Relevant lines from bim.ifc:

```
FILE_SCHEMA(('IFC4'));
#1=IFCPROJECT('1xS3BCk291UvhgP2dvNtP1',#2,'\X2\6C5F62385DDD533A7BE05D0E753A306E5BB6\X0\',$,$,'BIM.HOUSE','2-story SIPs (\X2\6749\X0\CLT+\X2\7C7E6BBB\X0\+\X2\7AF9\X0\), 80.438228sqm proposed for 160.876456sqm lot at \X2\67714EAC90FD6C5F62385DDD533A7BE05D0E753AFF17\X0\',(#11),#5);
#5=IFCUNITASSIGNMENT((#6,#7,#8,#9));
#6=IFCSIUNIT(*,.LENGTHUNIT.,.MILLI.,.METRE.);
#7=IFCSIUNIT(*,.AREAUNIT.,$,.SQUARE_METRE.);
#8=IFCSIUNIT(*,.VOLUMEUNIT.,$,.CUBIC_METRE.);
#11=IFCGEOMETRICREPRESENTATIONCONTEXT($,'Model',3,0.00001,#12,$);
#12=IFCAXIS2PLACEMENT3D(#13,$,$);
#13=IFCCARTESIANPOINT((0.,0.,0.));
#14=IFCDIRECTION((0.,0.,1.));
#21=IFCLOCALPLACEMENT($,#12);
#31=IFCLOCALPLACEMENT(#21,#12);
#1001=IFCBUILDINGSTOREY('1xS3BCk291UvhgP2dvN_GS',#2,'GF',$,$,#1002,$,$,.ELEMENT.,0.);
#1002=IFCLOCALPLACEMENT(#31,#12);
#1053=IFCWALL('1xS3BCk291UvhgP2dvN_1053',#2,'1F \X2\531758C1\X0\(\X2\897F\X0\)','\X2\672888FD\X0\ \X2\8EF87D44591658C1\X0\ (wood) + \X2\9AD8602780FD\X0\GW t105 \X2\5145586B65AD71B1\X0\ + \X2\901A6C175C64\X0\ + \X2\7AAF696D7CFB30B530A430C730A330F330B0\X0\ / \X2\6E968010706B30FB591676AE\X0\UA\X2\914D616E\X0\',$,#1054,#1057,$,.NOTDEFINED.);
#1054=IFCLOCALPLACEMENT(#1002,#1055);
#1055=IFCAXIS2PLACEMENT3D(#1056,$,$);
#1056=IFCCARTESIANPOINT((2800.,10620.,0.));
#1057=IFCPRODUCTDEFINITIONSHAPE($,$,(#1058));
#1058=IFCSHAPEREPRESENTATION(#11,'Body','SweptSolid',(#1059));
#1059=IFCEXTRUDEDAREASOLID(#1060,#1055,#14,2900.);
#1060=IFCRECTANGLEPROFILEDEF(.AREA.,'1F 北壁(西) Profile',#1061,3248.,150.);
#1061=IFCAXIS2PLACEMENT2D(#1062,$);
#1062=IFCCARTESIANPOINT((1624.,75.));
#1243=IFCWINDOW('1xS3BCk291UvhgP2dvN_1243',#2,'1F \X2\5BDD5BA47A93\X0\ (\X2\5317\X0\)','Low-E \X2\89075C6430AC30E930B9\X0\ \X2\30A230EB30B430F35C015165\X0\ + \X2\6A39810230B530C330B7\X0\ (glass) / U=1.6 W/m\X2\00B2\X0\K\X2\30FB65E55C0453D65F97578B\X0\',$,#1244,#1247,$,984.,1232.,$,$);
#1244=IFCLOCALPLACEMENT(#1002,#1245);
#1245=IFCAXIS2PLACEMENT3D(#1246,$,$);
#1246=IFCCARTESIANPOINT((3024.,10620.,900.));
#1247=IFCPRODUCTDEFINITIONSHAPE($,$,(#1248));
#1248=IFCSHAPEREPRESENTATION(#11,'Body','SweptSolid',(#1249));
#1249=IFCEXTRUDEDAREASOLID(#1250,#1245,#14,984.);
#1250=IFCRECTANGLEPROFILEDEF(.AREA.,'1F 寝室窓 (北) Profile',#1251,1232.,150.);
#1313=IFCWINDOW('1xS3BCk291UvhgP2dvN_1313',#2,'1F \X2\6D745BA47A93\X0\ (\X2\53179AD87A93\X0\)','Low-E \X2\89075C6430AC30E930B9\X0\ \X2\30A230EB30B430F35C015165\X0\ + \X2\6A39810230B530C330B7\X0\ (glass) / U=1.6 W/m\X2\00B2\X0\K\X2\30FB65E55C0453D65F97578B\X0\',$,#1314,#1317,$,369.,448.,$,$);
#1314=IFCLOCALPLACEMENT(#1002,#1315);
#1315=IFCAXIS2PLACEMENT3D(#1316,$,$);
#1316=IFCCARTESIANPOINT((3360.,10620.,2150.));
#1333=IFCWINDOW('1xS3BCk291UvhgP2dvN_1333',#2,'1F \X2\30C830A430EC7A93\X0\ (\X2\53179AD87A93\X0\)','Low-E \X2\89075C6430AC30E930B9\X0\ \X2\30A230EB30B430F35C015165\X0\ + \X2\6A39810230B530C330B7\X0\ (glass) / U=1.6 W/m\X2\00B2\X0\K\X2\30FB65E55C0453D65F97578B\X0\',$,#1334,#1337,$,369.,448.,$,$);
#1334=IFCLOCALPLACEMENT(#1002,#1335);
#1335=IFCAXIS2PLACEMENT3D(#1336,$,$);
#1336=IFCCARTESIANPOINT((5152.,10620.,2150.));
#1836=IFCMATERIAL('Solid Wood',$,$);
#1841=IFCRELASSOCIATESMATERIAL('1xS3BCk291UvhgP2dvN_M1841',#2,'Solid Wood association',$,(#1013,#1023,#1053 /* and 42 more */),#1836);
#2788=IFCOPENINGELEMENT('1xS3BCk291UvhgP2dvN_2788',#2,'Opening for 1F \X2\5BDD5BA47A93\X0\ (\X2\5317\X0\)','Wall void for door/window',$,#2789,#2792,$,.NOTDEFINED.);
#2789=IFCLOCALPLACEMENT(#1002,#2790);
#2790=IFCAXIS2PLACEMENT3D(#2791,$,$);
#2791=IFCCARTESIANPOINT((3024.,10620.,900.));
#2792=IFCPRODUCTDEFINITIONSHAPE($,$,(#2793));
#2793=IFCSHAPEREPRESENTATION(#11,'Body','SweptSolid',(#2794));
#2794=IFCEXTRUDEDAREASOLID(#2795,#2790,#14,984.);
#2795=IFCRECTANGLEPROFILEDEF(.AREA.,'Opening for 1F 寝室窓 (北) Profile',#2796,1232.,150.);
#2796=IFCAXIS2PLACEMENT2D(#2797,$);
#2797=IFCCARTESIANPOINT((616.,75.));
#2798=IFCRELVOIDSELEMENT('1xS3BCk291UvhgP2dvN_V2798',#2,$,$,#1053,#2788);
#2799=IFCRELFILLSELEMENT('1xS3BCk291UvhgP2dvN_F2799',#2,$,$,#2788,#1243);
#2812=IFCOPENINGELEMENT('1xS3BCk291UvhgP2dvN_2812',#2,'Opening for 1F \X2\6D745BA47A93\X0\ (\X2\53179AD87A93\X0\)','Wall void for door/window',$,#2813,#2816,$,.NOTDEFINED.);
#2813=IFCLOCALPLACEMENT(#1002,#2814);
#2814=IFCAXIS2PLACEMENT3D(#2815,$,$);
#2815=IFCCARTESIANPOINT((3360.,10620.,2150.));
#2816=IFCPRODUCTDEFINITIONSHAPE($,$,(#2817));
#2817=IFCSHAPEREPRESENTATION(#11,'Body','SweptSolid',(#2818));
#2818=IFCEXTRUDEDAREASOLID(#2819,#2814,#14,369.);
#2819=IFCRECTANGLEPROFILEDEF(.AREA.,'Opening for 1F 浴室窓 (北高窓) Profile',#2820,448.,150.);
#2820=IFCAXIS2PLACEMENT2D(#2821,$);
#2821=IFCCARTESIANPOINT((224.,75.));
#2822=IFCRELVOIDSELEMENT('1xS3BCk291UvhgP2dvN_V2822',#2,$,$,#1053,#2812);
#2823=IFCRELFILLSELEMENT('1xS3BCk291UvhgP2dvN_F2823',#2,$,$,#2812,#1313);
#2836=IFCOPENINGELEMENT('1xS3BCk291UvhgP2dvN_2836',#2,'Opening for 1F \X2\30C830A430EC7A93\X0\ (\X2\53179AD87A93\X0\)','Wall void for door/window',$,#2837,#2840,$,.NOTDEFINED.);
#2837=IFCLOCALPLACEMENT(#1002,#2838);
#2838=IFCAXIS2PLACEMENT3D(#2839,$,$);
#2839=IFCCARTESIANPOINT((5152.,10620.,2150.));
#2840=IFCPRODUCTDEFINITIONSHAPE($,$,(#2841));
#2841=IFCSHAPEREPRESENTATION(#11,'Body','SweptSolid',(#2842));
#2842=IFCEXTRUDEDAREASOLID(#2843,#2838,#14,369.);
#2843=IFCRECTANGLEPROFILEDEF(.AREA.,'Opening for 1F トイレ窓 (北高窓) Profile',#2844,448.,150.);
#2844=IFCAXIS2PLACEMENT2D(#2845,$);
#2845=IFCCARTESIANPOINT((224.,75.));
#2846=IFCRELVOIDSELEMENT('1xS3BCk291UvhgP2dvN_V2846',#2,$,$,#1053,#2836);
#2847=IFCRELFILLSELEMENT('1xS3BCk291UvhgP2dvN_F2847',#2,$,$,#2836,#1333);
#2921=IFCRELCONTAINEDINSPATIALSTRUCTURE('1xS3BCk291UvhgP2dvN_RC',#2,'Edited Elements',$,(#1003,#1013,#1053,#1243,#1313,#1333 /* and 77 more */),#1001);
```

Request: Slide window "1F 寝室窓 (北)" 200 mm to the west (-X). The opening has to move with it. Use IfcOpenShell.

```python
import ifcopenshell
import ifcopenshell.api.geometry
import ifcopenshell.util.placement

model = ifcopenshell.open("bim.ifc")

window = model.by_guid("1xS3BCk291UvhgP2dvN_1243")
opening = window.FillsVoids[0].RelatingOpeningElement
wall = opening.VoidsElements[0].RelatingBuildingElement

wall_matrix = ifcopenshell.util.placement.get_local_placement(wall.ObjectPlacement)
shift = wall_matrix[:3, 0] * -200.0
before = ifcopenshell.util.placement.get_local_placement(window.ObjectPlacement)[:3, 3].copy()

# The window is not placed relative to its opening, so move both.
for product in (opening, window):
    matrix = ifcopenshell.util.placement.get_local_placement(product.ObjectPlacement)
    matrix[:3, 3] += shift
    ifcopenshell.api.geometry.edit_object_placement(model, product=product, matrix=matrix, is_si=False)

after = ifcopenshell.util.placement.get_local_placement(window.ObjectPlacement)[:3, 3]
print("window moved by", (after - before).round(3) + 0.0)

model.write("bim_rev.ifc")
```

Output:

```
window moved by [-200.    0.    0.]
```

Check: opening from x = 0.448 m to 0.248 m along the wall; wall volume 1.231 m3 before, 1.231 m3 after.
